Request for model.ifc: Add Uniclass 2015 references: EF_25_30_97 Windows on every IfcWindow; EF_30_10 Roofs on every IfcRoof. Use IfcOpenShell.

First a look at what the model holds.

```python
import ifcopenshell

model = ifcopenshell.open("model.ifc")
print(model.schema)
print("classifications:", [c.Name for c in model.by_type("IfcClassification")])
for ifc_class in ("IfcDoor", "IfcRoof", "IfcStair", "IfcWall", "IfcWindow"):
    print(ifc_class, len(model.by_type(ifc_class)))
```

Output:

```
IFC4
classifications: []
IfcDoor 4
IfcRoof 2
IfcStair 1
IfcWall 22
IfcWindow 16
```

```python
import ifcopenshell
import ifcopenshell.api.classification

model = ifcopenshell.open("model.ifc")

system = ifcopenshell.api.classification.add_classification(model, classification="Uniclass 2015")

codes = {
    "IfcWindow": ("EF_25_30_97", "Windows"),
    "IfcRoof": ("EF_30_10", "Roofs"),
}
for ifc_class, (code, name) in codes.items():
    products = model.by_type(ifc_class)
    ifcopenshell.api.classification.add_reference(
        model, products=products, classification=system, identification=code, name=name
    )
    print(code, len(products))

model.write("model_updated.ifc")
```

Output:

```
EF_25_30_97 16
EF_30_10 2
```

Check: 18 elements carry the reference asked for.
